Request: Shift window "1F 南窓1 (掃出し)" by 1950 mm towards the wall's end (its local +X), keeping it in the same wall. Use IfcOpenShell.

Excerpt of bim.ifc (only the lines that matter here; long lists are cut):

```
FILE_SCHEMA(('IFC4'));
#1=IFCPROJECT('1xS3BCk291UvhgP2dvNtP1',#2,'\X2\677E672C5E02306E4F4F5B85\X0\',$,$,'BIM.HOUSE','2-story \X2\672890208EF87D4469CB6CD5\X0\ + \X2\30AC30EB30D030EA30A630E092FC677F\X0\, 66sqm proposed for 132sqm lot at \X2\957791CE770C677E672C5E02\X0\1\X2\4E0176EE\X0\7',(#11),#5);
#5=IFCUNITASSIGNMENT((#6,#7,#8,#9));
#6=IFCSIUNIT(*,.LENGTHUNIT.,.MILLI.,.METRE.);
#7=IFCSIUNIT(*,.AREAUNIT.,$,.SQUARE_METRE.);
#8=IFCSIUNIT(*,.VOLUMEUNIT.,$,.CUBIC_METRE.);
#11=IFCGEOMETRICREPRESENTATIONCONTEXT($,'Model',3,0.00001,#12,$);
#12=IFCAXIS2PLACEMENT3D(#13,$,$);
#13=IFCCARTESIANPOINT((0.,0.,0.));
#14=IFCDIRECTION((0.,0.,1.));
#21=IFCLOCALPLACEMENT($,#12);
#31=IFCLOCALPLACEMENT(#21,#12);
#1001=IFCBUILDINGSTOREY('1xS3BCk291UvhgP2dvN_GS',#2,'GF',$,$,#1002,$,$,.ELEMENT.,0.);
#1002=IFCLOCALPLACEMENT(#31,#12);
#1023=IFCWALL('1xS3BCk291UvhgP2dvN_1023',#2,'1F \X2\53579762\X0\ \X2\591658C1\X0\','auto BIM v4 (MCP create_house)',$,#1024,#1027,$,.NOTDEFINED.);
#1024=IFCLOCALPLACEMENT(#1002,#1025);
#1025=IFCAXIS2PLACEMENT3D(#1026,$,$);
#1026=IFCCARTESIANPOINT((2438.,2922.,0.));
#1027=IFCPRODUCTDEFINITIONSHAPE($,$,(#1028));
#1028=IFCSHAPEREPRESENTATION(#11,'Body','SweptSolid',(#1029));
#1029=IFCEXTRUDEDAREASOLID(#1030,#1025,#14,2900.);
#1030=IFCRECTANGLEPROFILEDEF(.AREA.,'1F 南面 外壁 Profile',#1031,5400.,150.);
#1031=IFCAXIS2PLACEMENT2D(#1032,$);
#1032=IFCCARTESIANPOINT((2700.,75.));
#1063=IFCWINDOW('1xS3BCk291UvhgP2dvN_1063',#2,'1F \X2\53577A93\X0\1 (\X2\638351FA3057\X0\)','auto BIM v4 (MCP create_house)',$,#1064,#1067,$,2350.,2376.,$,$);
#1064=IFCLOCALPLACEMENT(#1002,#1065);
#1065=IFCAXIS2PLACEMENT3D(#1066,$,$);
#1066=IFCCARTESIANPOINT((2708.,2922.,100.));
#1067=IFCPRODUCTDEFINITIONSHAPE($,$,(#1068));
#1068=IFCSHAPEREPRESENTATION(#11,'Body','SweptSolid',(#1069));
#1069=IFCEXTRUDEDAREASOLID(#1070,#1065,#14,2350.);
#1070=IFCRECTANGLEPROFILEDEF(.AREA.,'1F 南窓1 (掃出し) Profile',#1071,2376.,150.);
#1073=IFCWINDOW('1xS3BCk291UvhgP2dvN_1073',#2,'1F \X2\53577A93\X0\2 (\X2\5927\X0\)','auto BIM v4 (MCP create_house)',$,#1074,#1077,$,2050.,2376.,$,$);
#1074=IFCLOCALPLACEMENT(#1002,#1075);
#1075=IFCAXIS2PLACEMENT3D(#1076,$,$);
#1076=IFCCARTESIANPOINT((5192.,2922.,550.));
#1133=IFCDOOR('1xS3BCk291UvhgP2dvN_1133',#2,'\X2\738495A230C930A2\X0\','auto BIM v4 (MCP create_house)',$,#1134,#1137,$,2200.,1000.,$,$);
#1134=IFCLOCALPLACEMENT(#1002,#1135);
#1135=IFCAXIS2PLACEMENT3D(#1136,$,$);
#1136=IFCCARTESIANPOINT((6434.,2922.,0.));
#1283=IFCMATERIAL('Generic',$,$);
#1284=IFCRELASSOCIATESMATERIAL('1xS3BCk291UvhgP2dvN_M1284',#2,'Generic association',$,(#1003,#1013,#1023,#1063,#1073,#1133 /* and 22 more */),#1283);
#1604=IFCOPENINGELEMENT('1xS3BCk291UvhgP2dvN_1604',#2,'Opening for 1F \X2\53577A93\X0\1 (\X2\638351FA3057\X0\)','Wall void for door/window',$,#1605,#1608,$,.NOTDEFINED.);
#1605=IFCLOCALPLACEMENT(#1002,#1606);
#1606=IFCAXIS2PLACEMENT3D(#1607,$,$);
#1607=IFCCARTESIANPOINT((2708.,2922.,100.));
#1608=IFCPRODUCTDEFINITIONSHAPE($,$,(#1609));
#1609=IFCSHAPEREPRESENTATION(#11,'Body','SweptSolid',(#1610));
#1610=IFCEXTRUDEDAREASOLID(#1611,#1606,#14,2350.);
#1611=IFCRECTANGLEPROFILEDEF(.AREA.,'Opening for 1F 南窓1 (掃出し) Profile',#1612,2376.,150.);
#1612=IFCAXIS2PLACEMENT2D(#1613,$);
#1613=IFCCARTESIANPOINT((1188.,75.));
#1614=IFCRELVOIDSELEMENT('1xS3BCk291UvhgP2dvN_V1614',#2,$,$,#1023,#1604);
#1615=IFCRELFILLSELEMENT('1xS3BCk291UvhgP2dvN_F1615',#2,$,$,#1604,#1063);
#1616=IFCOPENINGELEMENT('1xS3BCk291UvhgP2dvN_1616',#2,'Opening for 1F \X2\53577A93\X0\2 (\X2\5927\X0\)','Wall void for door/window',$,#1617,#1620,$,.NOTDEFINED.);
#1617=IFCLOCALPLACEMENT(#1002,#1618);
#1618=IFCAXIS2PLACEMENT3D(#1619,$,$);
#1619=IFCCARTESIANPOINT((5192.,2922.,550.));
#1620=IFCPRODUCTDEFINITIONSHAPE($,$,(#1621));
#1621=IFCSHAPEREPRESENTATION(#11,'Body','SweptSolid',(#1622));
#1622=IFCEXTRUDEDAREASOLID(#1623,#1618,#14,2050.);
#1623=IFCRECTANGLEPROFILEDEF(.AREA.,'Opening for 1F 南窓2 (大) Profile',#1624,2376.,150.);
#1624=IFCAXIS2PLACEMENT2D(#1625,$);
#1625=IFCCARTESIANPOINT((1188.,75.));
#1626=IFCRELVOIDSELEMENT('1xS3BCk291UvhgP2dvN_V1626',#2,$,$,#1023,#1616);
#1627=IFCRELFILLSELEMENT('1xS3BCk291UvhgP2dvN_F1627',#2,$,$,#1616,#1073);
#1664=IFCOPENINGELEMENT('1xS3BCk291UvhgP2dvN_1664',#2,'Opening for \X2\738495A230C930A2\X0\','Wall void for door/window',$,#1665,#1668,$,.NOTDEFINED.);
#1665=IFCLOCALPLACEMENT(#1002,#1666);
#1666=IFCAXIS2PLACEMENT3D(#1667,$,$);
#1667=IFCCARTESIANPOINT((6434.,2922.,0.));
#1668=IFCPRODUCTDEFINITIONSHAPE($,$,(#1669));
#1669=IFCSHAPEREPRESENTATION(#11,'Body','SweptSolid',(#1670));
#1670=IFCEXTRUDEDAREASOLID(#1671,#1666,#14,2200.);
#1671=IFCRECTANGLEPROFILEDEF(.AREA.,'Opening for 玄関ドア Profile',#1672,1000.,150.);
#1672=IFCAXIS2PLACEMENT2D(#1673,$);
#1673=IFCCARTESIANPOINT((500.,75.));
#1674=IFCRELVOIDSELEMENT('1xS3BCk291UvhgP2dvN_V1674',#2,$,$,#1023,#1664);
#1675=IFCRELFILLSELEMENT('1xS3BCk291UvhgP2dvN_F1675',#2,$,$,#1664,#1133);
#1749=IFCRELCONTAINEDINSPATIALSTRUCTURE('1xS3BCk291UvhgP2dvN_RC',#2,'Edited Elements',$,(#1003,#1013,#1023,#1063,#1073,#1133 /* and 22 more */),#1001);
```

```python
import ifcopenshell
import ifcopenshell.api.geometry
import ifcopenshell.util.placement
import ifcopenshell.util.unit

model = ifcopenshell.open("bim.ifc")
unit_scale = ifcopenshell.util.unit.calculate_unit_scale(model)

window = model.by_guid("1xS3BCk291UvhgP2dvN_1063")
opening = window.FillsVoids[0].RelatingOpeningElement
wall = opening.VoidsElements[0].RelatingBuildingElement

wall_matrix = ifcopenshell.util.placement.get_local_placement(wall.ObjectPlacement)
shift = wall_matrix[:3, 0] * 1.95 / unit_scale
before = ifcopenshell.util.placement.get_local_placement(window.ObjectPlacement)[:3, 3].copy()

# The window is not placed relative to its opening, so move both.
for product in (opening, window):
    matrix = ifcopenshell.util.placement.get_local_placement(product.ObjectPlacement)
    matrix[:3, 3] += shift
    ifcopenshell.api.geometry.edit_object_placement(model, product=product, matrix=matrix, is_si=False)

after = ifcopenshell.util.placement.get_local_placement(window.ObjectPlacement)[:3, 3]
print("window moved by", (after - before).round(3) + 0.0)

model.write("bim_edited.ifc")
```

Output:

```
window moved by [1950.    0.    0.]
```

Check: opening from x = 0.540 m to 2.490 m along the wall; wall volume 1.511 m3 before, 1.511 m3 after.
